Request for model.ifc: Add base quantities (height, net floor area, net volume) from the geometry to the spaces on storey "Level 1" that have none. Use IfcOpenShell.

First a look at what the model holds.

```python
import ifcopenshell
import ifcopenshell.util.element
import ifcopenshell.util.unit

model = ifcopenshell.open("model.ifc")
print(model.schema)
for unit_type in ("LENGTHUNIT", "AREAUNIT", "VOLUMEUNIT"):
    print(unit_type, ifcopenshell.util.unit.calculate_unit_scale(model, unit_type))
storey = next(s for s in model.by_type("IfcBuildingStorey") if s.Name == "Level 1")
spaces = [e for e in ifcopenshell.util.element.get_decomposition(storey) if e.is_a("IfcSpace")]
for e in sorted(spaces, key=lambda e: e.id()):
    print(e.id(), e.is_a(), e.Name, list(ifcopenshell.util.element.get_psets(e, qtos_only=True)), sep=" | ")
```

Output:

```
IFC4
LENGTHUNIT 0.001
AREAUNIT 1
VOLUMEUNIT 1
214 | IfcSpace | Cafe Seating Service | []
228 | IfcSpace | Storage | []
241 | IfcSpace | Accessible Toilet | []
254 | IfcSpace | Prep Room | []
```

```python
import ifcopenshell
import ifcopenshell.api.pset
import ifcopenshell.geom
import ifcopenshell.util.element
import ifcopenshell.util.shape
import ifcopenshell.util.unit

model = ifcopenshell.open("model.ifc")
unit_scale = ifcopenshell.util.unit.calculate_unit_scale(model)
area_scale = ifcopenshell.util.unit.calculate_unit_scale(model, "AREAUNIT")
volume_scale = ifcopenshell.util.unit.calculate_unit_scale(model, "VOLUMEUNIT")
settings = ifcopenshell.geom.settings()

storey = next(s for s in model.by_type("IfcBuildingStorey") if s.Name == "Level 1")
spaces = [e for e in ifcopenshell.util.element.get_decomposition(storey) if e.is_a("IfcSpace")]

for e in sorted(spaces, key=lambda e: e.id()):
    if ifcopenshell.util.element.get_psets(e, qtos_only=True, should_inherit=False):
        continue
    # Geometry comes back in metres, in the element's own axes.
    shape = ifcopenshell.geom.create_shape(settings, e)
    values = {
        "Height": ifcopenshell.util.shape.get_z(shape.geometry) / unit_scale,
        "NetFloorArea": ifcopenshell.util.shape.get_footprint_area(shape.geometry) / area_scale,
        "NetVolume": ifcopenshell.util.shape.get_volume(shape.geometry) / volume_scale,
    }
    qto = ifcopenshell.api.pset.add_qto(model, product=e, name="Qto_SpaceBaseQuantities")
    ifcopenshell.api.pset.edit_qto(model, qto=qto, properties=values)
    print(e.id(), {k: round(v, 3) for k, v in values.items()})

model.write("model-out.ifc")
```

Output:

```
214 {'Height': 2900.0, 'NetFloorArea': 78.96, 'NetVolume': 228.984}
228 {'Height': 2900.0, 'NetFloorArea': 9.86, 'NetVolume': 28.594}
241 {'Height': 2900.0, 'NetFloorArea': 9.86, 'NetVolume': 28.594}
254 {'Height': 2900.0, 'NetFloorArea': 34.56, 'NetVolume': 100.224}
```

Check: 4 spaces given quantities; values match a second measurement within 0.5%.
